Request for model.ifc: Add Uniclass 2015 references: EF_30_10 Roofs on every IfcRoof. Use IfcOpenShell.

First a look at what the model holds.

```python
import ifcopenshell

model = ifcopenshell.open("model.ifc")
print(model.schema)
print("classifications:", [c.Name for c in model.by_type("IfcClassification")])
for ifc_class in ("IfcDoor", "IfcRoof", "IfcStair", "IfcWall", "IfcWindow"):
    print(ifc_class, len(model.by_type(ifc_class)))
```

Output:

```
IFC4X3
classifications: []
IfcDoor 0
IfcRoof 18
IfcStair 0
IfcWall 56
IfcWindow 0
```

```python
import ifcopenshell
import ifcopenshell.api.classification

model = ifcopenshell.open("model.ifc")

system = ifcopenshell.api.classification.add_classification(model, classification="Uniclass 2015")

codes = {
    "IfcRoof": ("EF_30_10", "Roofs"),
}
for ifc_class, (code, name) in codes.items():
    products = model.by_type(ifc_class)
    ifcopenshell.api.classification.add_reference(
        model, products=products, classification=system, identification=code, name=name
    )
    print(code, len(products))

model.write("model-out.ifc")
```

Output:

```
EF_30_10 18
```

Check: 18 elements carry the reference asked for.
